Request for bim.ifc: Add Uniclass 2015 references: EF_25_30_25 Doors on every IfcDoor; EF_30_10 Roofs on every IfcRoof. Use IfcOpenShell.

First a look at what the model holds.

```python
import ifcopenshell

model = ifcopenshell.open("bim.ifc")
print(model.schema)
print("classifications:", [c.Name for c in model.by_type("IfcClassification")])
for ifc_class in ("IfcDoor", "IfcRoof", "IfcStair", "IfcWall", "IfcWindow"):
    print(ifc_class, len(model.by_type(ifc_class)))
```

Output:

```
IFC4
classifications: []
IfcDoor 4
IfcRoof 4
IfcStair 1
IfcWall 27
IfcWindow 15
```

```python
import ifcopenshell
import ifcopenshell.api.classification

model = ifcopenshell.open("bim.ifc")

system = ifcopenshell.api.classification.add_classification(model, classification="Uniclass 2015")

codes = {
    "IfcDoor": ("EF_25_30_25", "Doors"),
    "IfcRoof": ("EF_30_10", "Roofs"),
}
for ifc_class, (code, name) in codes.items():
    products = model.by_type(ifc_class)
    ifcopenshell.api.classification.add_reference(
        model, products=products, classification=system, identification=code, name=name
    )
    print(code, len(products))

model.write("bim_updated.ifc")
```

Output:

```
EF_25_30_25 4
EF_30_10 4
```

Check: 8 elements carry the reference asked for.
